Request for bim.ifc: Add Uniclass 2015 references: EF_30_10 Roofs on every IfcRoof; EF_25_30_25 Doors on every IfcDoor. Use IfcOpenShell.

First a look at what the model holds.

```python
import ifcopenshell

model = ifcopenshell.open("bim.ifc")
print(model.schema)
print("classifications:", [c.Name for c in model.by_type("IfcClassification")])
for ifc_class in ("IfcDoor", "IfcRoof", "IfcStair", "IfcWall", "IfcWindow"):
    print(ifc_class, len(model.by_type(ifc_class)))
```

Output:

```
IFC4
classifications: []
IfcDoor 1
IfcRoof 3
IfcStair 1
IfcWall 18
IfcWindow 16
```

```python
import ifcopenshell
import ifcopenshell.api.classification

model = ifcopenshell.open("bim.ifc")

system = ifcopenshell.api.classification.add_classification(model, classification="Uniclass 2015")

codes = {
    "IfcRoof": ("EF_30_10", "Roofs"),
    "IfcDoor": ("EF_25_30_25", "Doors"),
}
for ifc_class, (code, name) in codes.items():
    products = model.by_type(ifc_class)
    ifcopenshell.api.classification.add_reference(
        model, products=products, classification=system, identification=code, name=name
    )
    print(code, len(products))

model.write("bim_rev.ifc")
```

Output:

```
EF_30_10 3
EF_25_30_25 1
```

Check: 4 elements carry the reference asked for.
